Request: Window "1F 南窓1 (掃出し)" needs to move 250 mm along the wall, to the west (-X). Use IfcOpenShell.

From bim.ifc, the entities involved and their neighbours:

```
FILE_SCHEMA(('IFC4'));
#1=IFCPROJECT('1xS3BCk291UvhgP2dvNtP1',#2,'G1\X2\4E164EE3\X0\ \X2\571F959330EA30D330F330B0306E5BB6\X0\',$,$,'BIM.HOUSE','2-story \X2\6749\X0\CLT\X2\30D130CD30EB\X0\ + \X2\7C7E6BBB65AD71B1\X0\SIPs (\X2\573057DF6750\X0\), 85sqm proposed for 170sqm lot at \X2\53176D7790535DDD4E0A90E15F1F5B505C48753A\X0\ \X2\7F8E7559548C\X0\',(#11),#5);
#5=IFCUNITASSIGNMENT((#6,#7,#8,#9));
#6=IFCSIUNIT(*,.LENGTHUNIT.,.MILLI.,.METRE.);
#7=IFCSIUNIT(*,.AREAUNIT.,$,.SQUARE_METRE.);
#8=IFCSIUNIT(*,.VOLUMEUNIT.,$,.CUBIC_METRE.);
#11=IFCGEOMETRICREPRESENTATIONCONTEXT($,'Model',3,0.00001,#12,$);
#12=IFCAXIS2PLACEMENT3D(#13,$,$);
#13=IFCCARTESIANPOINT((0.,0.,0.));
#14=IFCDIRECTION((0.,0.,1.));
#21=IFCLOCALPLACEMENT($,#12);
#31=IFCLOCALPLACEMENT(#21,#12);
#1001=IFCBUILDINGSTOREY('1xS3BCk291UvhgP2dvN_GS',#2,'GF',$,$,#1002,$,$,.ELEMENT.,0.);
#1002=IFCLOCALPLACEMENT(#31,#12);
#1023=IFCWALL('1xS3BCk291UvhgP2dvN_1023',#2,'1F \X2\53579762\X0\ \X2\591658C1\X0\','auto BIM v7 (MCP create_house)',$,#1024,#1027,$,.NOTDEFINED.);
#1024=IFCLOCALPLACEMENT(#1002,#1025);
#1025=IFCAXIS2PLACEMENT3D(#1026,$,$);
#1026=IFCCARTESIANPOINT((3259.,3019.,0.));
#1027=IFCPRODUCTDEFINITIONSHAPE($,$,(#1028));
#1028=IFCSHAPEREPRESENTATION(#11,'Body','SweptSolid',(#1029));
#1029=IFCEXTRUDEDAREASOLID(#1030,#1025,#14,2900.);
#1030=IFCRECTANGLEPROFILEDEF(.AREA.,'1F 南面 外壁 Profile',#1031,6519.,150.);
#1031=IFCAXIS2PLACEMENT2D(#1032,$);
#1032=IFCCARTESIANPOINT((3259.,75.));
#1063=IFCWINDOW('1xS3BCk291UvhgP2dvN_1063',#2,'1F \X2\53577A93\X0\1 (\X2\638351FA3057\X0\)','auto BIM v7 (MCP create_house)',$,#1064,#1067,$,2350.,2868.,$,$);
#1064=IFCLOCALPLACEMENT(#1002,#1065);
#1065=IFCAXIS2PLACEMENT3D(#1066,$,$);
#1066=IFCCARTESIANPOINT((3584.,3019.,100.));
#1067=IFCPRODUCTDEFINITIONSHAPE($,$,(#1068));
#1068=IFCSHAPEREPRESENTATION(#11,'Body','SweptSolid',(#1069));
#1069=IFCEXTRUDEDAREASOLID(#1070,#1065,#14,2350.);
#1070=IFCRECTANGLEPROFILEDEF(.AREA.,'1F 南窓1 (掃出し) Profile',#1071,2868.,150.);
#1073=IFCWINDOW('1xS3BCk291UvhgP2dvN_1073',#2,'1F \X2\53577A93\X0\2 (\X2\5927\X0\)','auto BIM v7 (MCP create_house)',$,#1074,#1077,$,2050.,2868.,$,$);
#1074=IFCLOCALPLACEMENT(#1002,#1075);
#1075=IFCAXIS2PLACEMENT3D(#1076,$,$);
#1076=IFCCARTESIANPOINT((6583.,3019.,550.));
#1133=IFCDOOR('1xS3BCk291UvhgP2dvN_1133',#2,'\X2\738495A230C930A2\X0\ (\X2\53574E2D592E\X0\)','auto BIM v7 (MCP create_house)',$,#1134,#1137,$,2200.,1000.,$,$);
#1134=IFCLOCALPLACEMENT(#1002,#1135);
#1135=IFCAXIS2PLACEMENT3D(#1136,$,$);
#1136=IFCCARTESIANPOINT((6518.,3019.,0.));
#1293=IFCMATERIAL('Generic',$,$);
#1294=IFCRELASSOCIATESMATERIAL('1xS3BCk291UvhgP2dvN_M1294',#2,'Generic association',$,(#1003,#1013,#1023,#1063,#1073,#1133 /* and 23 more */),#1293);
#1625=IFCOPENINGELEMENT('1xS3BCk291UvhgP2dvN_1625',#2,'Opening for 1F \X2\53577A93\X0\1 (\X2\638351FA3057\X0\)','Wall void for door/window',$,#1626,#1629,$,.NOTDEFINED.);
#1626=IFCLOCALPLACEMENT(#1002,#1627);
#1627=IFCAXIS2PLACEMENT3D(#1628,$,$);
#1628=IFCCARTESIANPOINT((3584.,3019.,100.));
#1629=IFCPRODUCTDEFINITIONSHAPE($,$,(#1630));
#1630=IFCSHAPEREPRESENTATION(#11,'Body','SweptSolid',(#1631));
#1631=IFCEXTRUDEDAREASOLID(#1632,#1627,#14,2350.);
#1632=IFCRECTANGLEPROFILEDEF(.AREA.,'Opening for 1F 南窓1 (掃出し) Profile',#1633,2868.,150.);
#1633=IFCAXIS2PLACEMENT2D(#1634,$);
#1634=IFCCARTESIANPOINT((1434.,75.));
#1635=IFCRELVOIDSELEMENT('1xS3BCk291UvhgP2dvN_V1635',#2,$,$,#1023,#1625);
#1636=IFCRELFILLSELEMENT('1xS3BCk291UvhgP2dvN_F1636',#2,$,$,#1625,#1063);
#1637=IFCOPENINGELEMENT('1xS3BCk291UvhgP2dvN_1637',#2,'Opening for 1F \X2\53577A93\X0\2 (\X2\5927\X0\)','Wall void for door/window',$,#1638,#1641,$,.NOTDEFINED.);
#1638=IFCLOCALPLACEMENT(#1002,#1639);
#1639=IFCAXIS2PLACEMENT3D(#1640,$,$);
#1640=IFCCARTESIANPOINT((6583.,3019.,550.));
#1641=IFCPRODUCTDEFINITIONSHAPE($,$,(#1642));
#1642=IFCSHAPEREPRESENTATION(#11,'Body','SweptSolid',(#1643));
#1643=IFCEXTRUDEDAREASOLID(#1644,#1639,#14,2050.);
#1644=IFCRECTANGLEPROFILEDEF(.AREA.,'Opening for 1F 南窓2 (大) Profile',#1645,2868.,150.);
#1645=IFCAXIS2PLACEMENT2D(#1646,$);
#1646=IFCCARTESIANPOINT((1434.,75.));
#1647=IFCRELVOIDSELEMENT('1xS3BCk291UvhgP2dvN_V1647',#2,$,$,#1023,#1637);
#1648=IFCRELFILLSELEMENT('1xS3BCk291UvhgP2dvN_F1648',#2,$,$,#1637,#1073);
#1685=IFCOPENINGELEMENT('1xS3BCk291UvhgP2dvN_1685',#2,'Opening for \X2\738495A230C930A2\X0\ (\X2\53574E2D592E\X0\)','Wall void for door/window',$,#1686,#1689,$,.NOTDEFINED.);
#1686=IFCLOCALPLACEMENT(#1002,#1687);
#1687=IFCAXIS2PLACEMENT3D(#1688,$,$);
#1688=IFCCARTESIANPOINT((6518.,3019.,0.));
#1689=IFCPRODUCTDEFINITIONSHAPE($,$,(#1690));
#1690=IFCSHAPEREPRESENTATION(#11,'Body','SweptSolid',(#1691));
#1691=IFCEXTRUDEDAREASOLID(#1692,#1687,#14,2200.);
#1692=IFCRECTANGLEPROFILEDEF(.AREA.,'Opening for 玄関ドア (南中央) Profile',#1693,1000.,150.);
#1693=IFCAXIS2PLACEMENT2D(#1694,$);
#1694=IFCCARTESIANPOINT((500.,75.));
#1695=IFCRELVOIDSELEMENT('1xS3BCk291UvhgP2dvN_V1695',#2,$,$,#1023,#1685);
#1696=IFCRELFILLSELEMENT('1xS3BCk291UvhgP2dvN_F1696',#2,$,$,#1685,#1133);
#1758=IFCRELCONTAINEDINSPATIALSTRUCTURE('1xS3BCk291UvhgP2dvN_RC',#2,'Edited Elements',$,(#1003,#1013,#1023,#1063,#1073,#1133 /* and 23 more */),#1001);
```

```python
import ifcopenshell
import ifcopenshell.api.geometry
import ifcopenshell.util.placement

model = ifcopenshell.open("bim.ifc")

window = model.by_guid("1xS3BCk291UvhgP2dvN_1063")
opening = window.FillsVoids[0].RelatingOpeningElement
wall = opening.VoidsElements[0].RelatingBuildingElement

wall_matrix = ifcopenshell.util.placement.get_local_placement(wall.ObjectPlacement)
shift = wall_matrix[:3, 0] * -250.0
before = ifcopenshell.util.placement.get_local_placement(window.ObjectPlacement)[:3, 3].copy()

# The window is not placed relative to its opening, so move both.
for product in (opening, window):
    matrix = ifcopenshell.util.placement.get_local_placement(product.ObjectPlacement)
    matrix[:3, 3] += shift
    ifcopenshell.api.geometry.edit_object_placement(model, product=product, matrix=matrix, is_si=False)

after = ifcopenshell.util.placement.get_local_placement(window.ObjectPlacement)[:3, 3]
print("window moved by", (after - before).round(3) + 0.0)

model.write("bim_updated.ifc")
```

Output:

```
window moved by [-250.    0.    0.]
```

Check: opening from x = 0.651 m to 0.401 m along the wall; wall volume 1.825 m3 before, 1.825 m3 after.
